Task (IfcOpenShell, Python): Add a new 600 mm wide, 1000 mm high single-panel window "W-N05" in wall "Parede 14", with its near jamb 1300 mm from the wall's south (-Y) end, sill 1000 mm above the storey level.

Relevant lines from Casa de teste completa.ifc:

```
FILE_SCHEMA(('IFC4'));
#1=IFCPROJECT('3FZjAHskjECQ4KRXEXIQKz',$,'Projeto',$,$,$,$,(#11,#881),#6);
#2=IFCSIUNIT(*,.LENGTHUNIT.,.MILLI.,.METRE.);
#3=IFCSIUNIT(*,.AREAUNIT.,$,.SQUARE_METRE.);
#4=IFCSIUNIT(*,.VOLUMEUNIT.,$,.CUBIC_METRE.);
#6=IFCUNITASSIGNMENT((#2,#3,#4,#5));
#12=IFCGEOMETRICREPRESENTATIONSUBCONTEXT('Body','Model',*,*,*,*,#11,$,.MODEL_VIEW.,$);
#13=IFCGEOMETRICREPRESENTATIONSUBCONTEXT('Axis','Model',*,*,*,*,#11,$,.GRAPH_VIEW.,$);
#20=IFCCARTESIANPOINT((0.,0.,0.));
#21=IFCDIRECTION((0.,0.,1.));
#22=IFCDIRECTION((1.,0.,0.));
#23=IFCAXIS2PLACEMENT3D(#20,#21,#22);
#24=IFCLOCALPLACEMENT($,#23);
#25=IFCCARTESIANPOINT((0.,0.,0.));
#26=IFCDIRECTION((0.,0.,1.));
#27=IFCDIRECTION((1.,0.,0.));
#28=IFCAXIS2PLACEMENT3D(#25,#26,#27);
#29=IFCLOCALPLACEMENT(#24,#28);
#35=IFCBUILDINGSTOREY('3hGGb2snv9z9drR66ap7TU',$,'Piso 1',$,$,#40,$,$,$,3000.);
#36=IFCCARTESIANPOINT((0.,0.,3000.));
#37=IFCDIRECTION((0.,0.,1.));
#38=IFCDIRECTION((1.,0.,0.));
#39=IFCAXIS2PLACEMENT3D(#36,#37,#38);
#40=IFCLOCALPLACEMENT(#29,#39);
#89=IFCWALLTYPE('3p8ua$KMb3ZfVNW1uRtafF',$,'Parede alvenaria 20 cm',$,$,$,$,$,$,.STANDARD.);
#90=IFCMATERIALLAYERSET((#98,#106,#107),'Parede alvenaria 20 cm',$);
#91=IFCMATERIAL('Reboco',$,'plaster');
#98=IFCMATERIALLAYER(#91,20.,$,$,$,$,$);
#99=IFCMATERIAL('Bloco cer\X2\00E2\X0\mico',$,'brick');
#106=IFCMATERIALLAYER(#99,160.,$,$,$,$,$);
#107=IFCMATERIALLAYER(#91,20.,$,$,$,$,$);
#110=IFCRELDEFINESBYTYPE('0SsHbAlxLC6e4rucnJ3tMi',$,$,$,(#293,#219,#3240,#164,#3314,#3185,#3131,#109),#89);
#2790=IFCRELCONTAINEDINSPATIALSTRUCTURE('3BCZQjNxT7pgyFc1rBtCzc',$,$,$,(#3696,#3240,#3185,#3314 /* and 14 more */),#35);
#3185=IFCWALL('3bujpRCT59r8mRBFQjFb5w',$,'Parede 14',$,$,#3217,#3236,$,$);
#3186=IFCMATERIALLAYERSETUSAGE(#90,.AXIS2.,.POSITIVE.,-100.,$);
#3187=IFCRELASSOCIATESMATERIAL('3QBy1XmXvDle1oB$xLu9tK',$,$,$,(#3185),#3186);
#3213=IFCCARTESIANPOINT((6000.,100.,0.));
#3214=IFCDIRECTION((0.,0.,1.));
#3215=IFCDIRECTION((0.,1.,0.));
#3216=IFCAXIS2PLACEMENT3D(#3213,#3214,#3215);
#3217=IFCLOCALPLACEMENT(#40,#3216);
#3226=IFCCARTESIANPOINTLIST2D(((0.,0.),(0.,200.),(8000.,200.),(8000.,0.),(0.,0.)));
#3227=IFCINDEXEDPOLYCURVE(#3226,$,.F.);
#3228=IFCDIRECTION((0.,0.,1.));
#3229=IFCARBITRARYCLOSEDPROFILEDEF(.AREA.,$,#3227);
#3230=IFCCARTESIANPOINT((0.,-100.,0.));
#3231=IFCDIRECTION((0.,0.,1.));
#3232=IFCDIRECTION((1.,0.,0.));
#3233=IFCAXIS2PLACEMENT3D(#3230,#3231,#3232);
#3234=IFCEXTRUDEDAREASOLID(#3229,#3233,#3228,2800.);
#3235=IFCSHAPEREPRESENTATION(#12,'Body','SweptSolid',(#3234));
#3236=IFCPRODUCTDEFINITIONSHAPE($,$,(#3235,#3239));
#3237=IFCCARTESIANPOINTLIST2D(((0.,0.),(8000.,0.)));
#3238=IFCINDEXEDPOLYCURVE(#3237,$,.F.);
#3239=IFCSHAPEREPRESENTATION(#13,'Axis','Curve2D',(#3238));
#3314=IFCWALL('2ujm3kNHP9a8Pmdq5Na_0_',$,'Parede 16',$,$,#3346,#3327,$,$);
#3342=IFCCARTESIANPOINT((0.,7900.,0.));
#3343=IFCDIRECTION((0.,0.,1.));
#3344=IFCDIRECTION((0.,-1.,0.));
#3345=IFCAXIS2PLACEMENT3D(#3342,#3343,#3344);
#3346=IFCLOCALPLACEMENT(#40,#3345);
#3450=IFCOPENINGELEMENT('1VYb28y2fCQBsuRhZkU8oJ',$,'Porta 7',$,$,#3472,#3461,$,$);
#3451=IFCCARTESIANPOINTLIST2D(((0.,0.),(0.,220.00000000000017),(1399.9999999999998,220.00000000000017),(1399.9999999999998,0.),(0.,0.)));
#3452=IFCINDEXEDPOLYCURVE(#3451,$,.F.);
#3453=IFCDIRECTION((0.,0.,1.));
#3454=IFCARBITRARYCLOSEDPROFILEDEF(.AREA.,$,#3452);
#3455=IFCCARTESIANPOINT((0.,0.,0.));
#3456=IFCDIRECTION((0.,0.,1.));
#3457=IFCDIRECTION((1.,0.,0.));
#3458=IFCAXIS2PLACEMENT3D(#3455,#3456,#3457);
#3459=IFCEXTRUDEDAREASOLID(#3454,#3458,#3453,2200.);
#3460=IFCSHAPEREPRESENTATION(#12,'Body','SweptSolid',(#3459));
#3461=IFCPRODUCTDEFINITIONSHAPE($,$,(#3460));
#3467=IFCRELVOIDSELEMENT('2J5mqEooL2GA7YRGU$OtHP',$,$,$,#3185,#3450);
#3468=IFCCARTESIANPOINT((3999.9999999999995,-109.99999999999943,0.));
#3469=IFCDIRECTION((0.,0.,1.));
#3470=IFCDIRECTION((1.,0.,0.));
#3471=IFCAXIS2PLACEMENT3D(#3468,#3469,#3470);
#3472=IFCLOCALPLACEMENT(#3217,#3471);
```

```python
import numpy as np
import ifcopenshell
import ifcopenshell.api.feature
import ifcopenshell.api.geometry
import ifcopenshell.api.root
import ifcopenshell.api.spatial
import ifcopenshell.geom
import ifcopenshell.util.element
import ifcopenshell.util.placement
import ifcopenshell.util.representation
import ifcopenshell.util.shape
import ifcopenshell.util.unit

model = ifcopenshell.open("Casa de teste completa.ifc")
unit_scale = ifcopenshell.util.unit.calculate_unit_scale(model)
settings = ifcopenshell.geom.settings()


def volume(element):
    """Net volume in cubic metres, openings subtracted."""
    shape = ifcopenshell.geom.create_shape(settings, element)
    return ifcopenshell.util.shape.get_volume(shape.geometry)


wall = model.by_guid("3bujpRCT59r8mRBFQjFb5w")
storey = ifcopenshell.util.element.get_container(wall, ifc_class="IfcBuildingStorey")
context = ifcopenshell.util.representation.get_context(model, "Model", "Body", "MODEL_VIEW")
before = volume(wall)

width, height, from_end, sill = 0.6, 1, 1.3, 1  # metres

# The wall runs along its own X axis, and the end named is its -X end.
wall_shape = ifcopenshell.geom.create_shape(settings, wall)
x, y, z = ifcopenshell.util.shape.get_vertices(wall_shape.geometry).T
start = x.min() + from_end
face, thickness = float(y.min()), float(y.max() - y.min())
wall_matrix = ifcopenshell.util.placement.get_local_placement(wall.ObjectPlacement)
level = ifcopenshell.util.placement.get_local_placement(storey.ObjectPlacement)[2, 3]


def in_wall(x, y):
    """Placement at x, y metres in the wall's axes, at sill height."""
    matrix = wall_matrix.copy()
    matrix[:, 3] = wall_matrix @ np.array([x / unit_scale, y / unit_scale, 0.0, 1.0])
    matrix[2, 3] = level + sill / unit_scale
    return matrix


# Opening: a box that overshoots both wall faces by 50 mm.
opening = ifcopenshell.api.root.create_entity(model, ifc_class="IfcOpeningElement", predefined_type="OPENING")
box = ifcopenshell.api.geometry.add_wall_representation(
    model, context=context, length=width, height=height, thickness=thickness + 0.1
)
ifcopenshell.api.geometry.assign_representation(model, product=opening, representation=box)
ifcopenshell.api.geometry.edit_object_placement(model, product=opening, matrix=in_wall(start, face - 0.05), is_si=False)
ifcopenshell.api.feature.add_feature(model, feature=opening, element=wall)

window = ifcopenshell.api.root.create_entity(model, ifc_class="IfcWindow", name="W-N05", predefined_type="WINDOW")
window.OverallWidth, window.OverallHeight = width / unit_scale, height / unit_scale
window.PartitioningType = "SINGLE_PANEL"
body = ifcopenshell.api.geometry.add_window_representation(
    model,
    context=context,
    overall_width=window.OverallWidth,
    overall_height=window.OverallHeight,
    partition_type="SINGLE_PANEL",
)
ifcopenshell.api.geometry.assign_representation(model, product=window, representation=body)
ifcopenshell.api.spatial.assign_container(model, products=[window], relating_structure=storey)
ifcopenshell.api.feature.add_filling(model, opening=opening, element=window)

# Centre the window in the wall's thickness.
ifcopenshell.api.geometry.edit_object_placement(model, product=window, matrix=in_wall(start, face), is_si=False)
window_shape = ifcopenshell.geom.create_shape(settings, window)
depth = ifcopenshell.util.shape.get_vertices(window_shape.geometry)[:, 1]
offset = face + thickness / 2 - (depth.min() + depth.max()) / 2
ifcopenshell.api.geometry.edit_object_placement(model, product=window, matrix=in_wall(start, offset), is_si=False)

after = volume(wall)

print(f"wall volume {before:.3f} -> {after:.3f} m3")

model.write("Casa de teste completa_updated.ifc")
```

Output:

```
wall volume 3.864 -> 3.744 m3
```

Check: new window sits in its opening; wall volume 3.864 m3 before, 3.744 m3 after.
